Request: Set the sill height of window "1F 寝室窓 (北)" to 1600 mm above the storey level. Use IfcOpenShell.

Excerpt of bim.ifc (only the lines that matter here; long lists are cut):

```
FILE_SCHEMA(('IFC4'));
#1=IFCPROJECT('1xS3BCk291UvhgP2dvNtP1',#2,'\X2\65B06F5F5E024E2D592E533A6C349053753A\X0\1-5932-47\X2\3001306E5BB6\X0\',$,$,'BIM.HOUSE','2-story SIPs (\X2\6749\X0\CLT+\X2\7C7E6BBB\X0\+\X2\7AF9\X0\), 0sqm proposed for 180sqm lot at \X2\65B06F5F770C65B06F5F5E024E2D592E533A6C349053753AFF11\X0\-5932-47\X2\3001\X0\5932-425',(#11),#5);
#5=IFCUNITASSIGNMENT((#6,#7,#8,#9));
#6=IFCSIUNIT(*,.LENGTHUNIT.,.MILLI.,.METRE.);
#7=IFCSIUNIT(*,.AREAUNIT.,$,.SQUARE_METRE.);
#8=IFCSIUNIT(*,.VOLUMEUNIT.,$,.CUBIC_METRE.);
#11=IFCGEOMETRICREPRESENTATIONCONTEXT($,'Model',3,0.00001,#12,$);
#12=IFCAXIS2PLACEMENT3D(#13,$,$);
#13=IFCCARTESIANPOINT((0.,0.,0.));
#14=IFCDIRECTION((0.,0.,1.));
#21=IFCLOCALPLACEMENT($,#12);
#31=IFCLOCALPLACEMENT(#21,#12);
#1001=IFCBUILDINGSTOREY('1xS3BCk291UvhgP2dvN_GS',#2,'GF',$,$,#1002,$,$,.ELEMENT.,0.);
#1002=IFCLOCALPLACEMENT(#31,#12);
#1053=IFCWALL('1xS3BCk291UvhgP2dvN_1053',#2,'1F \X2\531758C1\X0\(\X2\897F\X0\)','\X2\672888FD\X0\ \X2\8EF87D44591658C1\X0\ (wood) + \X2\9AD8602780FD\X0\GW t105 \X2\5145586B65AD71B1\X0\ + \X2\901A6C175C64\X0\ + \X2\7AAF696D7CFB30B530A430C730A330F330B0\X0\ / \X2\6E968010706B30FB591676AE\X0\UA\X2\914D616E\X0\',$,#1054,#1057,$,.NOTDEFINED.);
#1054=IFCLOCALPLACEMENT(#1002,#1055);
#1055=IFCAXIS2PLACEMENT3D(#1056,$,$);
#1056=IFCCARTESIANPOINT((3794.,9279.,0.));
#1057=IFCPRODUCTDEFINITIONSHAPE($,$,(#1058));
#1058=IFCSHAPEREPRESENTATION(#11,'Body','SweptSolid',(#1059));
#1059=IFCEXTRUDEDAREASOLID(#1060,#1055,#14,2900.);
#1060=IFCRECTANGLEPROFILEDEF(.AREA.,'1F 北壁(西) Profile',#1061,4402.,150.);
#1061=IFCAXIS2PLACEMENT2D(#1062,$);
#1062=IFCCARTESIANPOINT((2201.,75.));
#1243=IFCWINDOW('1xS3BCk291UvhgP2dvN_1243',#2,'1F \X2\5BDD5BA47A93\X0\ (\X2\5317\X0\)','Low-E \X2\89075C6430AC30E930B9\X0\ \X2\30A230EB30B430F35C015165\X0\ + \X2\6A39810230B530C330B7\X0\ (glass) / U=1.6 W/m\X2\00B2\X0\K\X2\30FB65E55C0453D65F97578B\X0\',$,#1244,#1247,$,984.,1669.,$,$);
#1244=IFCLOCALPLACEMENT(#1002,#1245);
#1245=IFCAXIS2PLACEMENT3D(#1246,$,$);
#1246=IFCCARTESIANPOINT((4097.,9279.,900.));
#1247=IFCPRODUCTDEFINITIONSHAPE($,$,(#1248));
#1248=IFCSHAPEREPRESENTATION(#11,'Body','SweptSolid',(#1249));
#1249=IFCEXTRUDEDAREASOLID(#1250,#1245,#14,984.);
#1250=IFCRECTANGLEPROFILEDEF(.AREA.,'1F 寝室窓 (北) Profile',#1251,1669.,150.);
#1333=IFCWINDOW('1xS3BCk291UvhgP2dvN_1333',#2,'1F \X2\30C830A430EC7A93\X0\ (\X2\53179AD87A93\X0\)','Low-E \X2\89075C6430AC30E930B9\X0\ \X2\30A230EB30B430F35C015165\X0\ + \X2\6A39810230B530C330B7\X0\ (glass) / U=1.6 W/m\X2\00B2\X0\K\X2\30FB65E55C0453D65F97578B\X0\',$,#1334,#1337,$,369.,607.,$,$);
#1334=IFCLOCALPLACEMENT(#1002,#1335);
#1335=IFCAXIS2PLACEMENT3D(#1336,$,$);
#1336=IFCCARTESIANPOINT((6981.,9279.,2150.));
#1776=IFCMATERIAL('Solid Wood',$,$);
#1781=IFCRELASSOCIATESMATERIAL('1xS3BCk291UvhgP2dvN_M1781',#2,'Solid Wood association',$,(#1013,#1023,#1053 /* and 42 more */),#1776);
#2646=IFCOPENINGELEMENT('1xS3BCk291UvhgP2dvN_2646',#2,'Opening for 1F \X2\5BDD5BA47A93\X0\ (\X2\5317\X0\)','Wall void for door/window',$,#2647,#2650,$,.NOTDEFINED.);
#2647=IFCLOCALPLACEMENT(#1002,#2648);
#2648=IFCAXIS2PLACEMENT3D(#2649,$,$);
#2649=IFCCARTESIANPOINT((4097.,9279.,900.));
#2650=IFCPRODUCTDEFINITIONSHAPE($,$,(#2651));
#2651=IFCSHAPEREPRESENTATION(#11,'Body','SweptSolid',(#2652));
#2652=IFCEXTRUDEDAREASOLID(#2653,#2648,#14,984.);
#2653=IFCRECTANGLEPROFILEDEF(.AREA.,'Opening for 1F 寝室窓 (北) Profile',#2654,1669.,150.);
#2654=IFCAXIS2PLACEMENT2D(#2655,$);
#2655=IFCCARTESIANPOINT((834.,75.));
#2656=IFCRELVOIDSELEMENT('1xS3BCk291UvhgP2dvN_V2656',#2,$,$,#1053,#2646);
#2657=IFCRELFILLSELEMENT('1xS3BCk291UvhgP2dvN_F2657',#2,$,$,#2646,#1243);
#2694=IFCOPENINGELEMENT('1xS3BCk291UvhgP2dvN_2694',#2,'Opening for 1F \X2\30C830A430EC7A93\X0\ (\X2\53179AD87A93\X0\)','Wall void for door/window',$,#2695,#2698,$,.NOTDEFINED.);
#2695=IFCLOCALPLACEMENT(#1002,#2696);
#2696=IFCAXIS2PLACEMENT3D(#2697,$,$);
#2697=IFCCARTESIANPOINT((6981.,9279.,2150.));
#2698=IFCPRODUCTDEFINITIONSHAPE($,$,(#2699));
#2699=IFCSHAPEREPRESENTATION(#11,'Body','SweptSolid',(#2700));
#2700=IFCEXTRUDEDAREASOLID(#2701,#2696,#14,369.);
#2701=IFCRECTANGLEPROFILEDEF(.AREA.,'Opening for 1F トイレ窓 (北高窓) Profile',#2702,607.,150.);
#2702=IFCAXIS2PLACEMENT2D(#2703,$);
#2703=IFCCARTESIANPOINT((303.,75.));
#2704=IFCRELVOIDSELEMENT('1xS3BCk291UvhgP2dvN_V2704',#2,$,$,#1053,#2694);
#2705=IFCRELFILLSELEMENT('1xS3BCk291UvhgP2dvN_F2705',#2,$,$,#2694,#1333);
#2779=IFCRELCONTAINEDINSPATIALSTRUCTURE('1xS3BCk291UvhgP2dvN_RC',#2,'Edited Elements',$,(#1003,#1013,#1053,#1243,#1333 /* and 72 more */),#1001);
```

```python
import numpy as np
import ifcopenshell
import ifcopenshell.api.geometry
import ifcopenshell.geom
import ifcopenshell.util.element
import ifcopenshell.util.placement
import ifcopenshell.util.shape
import ifcopenshell.util.unit

model = ifcopenshell.open("bim.ifc")
unit_scale = ifcopenshell.util.unit.calculate_unit_scale(model)

window = model.by_guid("1xS3BCk291UvhgP2dvN_1243")
opening = window.FillsVoids[0].RelatingOpeningElement
storey = ifcopenshell.util.element.get_container(window, ifc_class="IfcBuildingStorey")
level = ifcopenshell.util.placement.get_local_placement(storey.ObjectPlacement)[2, 3]

# The opening's origin need not be at the sill, so measure its lowest point.
shape = ifcopenshell.geom.create_shape(ifcopenshell.geom.settings(), opening)
bottom = ifcopenshell.util.shape.get_shape_bottom_elevation(shape, shape.geometry) / unit_scale
dz = level + 1.6 / unit_scale - bottom

shift = np.array([0.0, 0.0, dz])
# The window is not placed relative to its opening, so move both.
for product in (opening, window):
    matrix = ifcopenshell.util.placement.get_local_placement(product.ObjectPlacement)
    matrix[:3, 3] += shift
    ifcopenshell.api.geometry.edit_object_placement(model, product=product, matrix=matrix, is_si=False)

print(f"moved by {dz * unit_scale:+.3f} m")

model.write("bim_edited.ifc")
```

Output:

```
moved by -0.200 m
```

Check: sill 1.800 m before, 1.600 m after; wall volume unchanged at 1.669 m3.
